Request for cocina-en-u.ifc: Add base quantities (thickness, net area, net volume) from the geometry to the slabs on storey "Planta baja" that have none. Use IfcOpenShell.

First a look at what the model holds.

```python
import ifcopenshell
import ifcopenshell.util.element
import ifcopenshell.util.unit

model = ifcopenshell.open("cocina-en-u.ifc")
print(model.schema)
for unit_type in ("LENGTHUNIT", "AREAUNIT", "VOLUMEUNIT"):
    print(unit_type, ifcopenshell.util.unit.calculate_unit_scale(model, unit_type))
storey = next(s for s in model.by_type("IfcBuildingStorey") if s.Name == "Planta baja")
slabs = [e for e in ifcopenshell.util.element.get_decomposition(storey) if e.is_a("IfcSlab")]
for e in sorted(slabs, key=lambda e: e.id()):
    print(e.id(), e.is_a(), e.Name, list(ifcopenshell.util.element.get_psets(e, qtos_only=True)), sep=" | ")
```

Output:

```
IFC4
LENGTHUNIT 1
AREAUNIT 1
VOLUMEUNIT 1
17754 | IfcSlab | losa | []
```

```python
import ifcopenshell
import ifcopenshell.api.pset
import ifcopenshell.geom
import ifcopenshell.util.element
import ifcopenshell.util.shape
import ifcopenshell.util.unit

model = ifcopenshell.open("cocina-en-u.ifc")
unit_scale = ifcopenshell.util.unit.calculate_unit_scale(model)
area_scale = ifcopenshell.util.unit.calculate_unit_scale(model, "AREAUNIT")
volume_scale = ifcopenshell.util.unit.calculate_unit_scale(model, "VOLUMEUNIT")
settings = ifcopenshell.geom.settings()

storey = next(s for s in model.by_type("IfcBuildingStorey") if s.Name == "Planta baja")
slabs = [e for e in ifcopenshell.util.element.get_decomposition(storey) if e.is_a("IfcSlab")]

for e in sorted(slabs, key=lambda e: e.id()):
    if ifcopenshell.util.element.get_psets(e, qtos_only=True, should_inherit=False):
        continue
    # Geometry comes back in metres, in the element's own axes.
    shape = ifcopenshell.geom.create_shape(settings, e)
    values = {
        "Width": ifcopenshell.util.shape.get_z(shape.geometry) / unit_scale,
        "NetArea": ifcopenshell.util.shape.get_footprint_area(shape.geometry) / area_scale,
        "NetVolume": ifcopenshell.util.shape.get_volume(shape.geometry) / volume_scale,
    }
    qto = ifcopenshell.api.pset.add_qto(model, product=e, name="Qto_SlabBaseQuantities")
    ifcopenshell.api.pset.edit_qto(model, qto=qto, properties=values)
    print(e.id(), {k: round(v, 3) for k, v in values.items()})

model.write("cocina-en-u_updated.ifc")
```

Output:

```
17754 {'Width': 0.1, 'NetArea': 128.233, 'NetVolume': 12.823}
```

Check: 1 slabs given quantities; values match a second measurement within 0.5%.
